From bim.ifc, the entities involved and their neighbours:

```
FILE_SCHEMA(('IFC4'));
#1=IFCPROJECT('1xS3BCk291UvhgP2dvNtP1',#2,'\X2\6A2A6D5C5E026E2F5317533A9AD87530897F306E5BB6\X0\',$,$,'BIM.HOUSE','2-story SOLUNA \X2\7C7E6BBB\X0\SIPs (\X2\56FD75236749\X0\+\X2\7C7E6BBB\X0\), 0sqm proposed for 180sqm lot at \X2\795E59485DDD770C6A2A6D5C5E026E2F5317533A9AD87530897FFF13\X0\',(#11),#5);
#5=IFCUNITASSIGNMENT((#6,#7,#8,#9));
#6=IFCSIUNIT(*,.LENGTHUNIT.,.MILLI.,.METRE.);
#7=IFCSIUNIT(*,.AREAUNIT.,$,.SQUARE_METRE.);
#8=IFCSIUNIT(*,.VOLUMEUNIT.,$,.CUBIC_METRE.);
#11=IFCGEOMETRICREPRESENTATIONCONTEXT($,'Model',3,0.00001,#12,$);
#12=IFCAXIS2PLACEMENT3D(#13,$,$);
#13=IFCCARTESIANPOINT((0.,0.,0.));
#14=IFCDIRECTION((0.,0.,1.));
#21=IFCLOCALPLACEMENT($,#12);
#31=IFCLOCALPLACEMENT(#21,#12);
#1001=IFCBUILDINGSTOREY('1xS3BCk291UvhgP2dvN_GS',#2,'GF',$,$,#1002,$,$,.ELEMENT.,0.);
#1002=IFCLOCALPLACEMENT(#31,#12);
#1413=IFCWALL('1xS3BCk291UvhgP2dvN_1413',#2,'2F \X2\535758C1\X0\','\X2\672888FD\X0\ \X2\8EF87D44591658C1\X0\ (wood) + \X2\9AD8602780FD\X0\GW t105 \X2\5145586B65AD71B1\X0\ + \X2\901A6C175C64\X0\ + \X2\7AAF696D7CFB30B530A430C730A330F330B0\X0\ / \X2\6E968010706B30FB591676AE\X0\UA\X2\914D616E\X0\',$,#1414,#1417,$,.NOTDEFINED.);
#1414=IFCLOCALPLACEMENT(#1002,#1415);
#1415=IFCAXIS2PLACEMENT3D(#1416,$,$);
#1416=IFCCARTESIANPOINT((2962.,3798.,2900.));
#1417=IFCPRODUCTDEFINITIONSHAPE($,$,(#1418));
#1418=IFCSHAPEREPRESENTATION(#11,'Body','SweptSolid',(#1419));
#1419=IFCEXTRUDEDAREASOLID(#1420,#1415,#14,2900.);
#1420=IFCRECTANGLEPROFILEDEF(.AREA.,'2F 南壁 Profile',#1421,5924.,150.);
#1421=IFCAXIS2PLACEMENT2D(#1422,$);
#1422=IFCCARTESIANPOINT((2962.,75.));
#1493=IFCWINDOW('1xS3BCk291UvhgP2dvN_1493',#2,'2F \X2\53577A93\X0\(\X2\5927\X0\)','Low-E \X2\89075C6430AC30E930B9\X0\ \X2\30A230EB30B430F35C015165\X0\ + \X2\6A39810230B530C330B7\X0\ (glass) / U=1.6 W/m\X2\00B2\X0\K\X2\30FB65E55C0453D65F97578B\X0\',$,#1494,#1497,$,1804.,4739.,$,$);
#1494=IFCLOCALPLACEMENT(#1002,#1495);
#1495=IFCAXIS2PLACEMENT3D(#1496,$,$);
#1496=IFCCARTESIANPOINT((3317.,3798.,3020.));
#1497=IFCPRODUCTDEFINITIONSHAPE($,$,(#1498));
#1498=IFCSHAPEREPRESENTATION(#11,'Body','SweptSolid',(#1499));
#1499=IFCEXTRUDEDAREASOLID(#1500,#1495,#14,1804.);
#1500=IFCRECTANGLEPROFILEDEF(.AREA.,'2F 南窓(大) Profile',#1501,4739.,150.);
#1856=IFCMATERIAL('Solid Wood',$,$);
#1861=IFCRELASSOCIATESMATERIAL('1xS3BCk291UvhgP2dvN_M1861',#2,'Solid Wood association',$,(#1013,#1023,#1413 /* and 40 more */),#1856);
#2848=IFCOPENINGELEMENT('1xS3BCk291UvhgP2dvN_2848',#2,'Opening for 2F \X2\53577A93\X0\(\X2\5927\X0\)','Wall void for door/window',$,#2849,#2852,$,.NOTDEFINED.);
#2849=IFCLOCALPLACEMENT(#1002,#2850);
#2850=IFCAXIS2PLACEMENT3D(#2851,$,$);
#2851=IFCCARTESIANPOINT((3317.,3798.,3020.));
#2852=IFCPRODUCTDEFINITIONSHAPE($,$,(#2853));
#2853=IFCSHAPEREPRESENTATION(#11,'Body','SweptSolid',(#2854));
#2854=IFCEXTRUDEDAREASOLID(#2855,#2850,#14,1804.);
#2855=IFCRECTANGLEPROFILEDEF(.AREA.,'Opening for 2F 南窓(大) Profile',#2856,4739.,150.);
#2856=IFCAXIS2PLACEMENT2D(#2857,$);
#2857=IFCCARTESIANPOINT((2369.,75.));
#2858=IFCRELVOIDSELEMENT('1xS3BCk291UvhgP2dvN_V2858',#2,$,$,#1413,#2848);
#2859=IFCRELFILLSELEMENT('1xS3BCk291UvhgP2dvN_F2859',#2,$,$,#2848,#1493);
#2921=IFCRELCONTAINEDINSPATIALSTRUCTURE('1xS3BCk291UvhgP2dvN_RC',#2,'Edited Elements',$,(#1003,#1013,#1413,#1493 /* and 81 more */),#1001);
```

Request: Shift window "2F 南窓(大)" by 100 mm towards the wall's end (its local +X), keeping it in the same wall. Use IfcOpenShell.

```python
import ifcopenshell
import ifcopenshell.api.geometry
import ifcopenshell.util.placement

model = ifcopenshell.open("bim.ifc")

window = model.by_id(1493)
opening = window.FillsVoids[0].RelatingOpeningElement
wall = opening.VoidsElements[0].RelatingBuildingElement

wall_matrix = ifcopenshell.util.placement.get_local_placement(wall.ObjectPlacement)
shift = wall_matrix[:3, 0] * 100.0
before = ifcopenshell.util.placement.get_local_placement(window.ObjectPlacement)[:3, 3].copy()

# The window is not placed relative to its opening, so move both.
for product in (opening, window):
    matrix = ifcopenshell.util.placement.get_local_placement(product.ObjectPlacement)
    matrix[:3, 3] += shift
    ifcopenshell.api.geometry.edit_object_placement(model, product=product, matrix=matrix, is_si=False)

after = ifcopenshell.util.placement.get_local_placement(window.ObjectPlacement)[:3, 3]
print("window moved by", (after - before).round(3) + 0.0)

model.write("bim_updated.ifc")
```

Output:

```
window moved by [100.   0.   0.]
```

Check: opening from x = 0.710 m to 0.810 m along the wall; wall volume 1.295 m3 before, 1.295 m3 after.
